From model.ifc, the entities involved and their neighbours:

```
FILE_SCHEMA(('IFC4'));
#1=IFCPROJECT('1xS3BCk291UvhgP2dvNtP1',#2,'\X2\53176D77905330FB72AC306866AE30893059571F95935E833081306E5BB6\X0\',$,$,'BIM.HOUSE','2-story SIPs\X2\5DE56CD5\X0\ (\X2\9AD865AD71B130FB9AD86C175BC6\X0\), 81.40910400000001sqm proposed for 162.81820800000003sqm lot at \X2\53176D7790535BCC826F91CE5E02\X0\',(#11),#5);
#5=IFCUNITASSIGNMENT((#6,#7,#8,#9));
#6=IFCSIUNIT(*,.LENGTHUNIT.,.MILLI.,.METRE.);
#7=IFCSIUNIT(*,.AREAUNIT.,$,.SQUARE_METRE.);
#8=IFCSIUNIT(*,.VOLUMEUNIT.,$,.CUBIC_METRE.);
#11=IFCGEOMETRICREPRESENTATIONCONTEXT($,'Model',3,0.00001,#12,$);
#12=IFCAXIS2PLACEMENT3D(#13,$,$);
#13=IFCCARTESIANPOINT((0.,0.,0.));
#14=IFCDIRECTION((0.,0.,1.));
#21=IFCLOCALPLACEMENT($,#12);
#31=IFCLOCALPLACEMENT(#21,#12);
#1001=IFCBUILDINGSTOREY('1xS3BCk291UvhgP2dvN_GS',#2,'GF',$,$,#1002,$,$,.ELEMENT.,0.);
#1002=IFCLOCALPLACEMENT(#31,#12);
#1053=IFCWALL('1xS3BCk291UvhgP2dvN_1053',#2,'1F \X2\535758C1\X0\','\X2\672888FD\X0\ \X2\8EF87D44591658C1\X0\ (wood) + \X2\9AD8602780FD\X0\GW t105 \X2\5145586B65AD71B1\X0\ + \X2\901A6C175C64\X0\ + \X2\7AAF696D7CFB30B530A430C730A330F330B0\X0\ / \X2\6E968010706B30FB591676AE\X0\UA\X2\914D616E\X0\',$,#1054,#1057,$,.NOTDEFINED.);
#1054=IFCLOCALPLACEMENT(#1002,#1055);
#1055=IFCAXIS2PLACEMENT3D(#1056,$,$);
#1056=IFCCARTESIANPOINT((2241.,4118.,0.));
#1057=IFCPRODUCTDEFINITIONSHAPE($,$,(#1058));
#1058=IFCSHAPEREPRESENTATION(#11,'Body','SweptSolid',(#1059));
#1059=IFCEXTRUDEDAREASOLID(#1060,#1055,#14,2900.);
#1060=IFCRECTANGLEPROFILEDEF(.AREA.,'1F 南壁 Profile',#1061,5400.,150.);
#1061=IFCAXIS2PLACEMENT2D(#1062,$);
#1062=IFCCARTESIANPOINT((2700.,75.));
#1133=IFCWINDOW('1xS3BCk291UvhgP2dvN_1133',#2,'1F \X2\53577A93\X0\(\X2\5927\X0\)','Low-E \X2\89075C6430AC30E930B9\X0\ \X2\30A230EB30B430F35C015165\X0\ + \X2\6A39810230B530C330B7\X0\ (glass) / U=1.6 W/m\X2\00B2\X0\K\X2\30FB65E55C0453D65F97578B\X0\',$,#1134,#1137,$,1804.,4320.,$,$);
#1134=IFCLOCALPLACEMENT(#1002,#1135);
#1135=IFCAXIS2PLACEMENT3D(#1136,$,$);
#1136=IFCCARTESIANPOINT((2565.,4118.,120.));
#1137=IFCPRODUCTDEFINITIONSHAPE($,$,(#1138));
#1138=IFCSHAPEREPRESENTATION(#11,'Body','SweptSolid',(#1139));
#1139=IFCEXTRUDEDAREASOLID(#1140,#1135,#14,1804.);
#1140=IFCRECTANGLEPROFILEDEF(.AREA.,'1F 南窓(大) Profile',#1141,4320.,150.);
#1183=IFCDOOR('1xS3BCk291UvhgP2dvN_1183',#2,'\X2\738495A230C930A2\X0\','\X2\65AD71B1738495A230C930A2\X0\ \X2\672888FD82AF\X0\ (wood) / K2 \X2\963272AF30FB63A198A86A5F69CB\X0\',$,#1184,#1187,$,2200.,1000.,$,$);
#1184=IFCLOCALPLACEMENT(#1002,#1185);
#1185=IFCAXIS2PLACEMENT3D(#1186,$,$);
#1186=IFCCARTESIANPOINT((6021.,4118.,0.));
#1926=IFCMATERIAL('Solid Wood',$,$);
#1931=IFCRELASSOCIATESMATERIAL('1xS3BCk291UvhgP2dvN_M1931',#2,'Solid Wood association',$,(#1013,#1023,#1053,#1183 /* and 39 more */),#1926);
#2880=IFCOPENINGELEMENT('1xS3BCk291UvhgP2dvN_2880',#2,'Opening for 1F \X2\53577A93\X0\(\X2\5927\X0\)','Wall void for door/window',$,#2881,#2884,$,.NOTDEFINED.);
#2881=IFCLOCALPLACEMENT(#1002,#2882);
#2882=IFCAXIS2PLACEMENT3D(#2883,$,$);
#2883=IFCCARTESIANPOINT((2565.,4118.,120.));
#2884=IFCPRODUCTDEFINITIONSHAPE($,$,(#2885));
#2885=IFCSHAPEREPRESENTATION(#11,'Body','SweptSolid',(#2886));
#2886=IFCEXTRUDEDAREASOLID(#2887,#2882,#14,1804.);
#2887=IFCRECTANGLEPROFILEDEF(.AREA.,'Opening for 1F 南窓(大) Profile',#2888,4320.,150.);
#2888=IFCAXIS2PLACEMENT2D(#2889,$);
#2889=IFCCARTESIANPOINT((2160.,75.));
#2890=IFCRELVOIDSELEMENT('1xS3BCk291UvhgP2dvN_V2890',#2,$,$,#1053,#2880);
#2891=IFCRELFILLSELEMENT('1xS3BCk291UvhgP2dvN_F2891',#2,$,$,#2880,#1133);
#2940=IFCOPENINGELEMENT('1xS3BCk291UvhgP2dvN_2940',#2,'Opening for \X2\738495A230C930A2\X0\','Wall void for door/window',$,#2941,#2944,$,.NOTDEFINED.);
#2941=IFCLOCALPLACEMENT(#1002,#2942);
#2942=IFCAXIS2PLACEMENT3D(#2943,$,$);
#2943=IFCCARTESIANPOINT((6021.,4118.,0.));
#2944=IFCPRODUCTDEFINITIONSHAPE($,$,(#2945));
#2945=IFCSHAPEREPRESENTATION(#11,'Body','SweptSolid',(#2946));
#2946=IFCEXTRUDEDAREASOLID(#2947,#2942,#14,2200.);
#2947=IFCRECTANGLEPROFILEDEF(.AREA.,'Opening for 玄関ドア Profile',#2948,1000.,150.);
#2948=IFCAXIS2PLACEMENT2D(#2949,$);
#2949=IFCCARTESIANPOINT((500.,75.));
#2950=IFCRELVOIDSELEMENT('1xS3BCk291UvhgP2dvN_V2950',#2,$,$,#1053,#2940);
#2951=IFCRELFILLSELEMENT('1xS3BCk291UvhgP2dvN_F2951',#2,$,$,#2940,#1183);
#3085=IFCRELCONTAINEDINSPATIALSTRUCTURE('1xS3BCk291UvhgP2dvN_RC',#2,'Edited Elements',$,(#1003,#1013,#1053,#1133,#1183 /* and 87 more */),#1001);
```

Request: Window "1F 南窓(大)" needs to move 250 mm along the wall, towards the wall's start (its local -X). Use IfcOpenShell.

```python
import ifcopenshell
import ifcopenshell.api.geometry
import ifcopenshell.util.placement
import ifcopenshell.util.unit

model = ifcopenshell.open("model.ifc")
unit_scale = ifcopenshell.util.unit.calculate_unit_scale(model)

window = model.by_guid("1xS3BCk291UvhgP2dvN_1133")
opening = window.FillsVoids[0].RelatingOpeningElement
wall = opening.VoidsElements[0].RelatingBuildingElement

wall_matrix = ifcopenshell.util.placement.get_local_placement(wall.ObjectPlacement)
shift = wall_matrix[:3, 0] * -0.25 / unit_scale
before = ifcopenshell.util.placement.get_local_placement(window.ObjectPlacement)[:3, 3].copy()

# The window is not placed relative to its opening, so move both.
for product in (opening, window):
    matrix = ifcopenshell.util.placement.get_local_placement(product.ObjectPlacement)
    matrix[:3, 3] += shift
    ifcopenshell.api.geometry.edit_object_placement(model, product=product, matrix=matrix, is_si=False)

after = ifcopenshell.util.placement.get_local_placement(window.ObjectPlacement)[:3, 3]
print("window moved by", (after - before).round(3) + 0.0)

model.write("model_v2.ifc")
```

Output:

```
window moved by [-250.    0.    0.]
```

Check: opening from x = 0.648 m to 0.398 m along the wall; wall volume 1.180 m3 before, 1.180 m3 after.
